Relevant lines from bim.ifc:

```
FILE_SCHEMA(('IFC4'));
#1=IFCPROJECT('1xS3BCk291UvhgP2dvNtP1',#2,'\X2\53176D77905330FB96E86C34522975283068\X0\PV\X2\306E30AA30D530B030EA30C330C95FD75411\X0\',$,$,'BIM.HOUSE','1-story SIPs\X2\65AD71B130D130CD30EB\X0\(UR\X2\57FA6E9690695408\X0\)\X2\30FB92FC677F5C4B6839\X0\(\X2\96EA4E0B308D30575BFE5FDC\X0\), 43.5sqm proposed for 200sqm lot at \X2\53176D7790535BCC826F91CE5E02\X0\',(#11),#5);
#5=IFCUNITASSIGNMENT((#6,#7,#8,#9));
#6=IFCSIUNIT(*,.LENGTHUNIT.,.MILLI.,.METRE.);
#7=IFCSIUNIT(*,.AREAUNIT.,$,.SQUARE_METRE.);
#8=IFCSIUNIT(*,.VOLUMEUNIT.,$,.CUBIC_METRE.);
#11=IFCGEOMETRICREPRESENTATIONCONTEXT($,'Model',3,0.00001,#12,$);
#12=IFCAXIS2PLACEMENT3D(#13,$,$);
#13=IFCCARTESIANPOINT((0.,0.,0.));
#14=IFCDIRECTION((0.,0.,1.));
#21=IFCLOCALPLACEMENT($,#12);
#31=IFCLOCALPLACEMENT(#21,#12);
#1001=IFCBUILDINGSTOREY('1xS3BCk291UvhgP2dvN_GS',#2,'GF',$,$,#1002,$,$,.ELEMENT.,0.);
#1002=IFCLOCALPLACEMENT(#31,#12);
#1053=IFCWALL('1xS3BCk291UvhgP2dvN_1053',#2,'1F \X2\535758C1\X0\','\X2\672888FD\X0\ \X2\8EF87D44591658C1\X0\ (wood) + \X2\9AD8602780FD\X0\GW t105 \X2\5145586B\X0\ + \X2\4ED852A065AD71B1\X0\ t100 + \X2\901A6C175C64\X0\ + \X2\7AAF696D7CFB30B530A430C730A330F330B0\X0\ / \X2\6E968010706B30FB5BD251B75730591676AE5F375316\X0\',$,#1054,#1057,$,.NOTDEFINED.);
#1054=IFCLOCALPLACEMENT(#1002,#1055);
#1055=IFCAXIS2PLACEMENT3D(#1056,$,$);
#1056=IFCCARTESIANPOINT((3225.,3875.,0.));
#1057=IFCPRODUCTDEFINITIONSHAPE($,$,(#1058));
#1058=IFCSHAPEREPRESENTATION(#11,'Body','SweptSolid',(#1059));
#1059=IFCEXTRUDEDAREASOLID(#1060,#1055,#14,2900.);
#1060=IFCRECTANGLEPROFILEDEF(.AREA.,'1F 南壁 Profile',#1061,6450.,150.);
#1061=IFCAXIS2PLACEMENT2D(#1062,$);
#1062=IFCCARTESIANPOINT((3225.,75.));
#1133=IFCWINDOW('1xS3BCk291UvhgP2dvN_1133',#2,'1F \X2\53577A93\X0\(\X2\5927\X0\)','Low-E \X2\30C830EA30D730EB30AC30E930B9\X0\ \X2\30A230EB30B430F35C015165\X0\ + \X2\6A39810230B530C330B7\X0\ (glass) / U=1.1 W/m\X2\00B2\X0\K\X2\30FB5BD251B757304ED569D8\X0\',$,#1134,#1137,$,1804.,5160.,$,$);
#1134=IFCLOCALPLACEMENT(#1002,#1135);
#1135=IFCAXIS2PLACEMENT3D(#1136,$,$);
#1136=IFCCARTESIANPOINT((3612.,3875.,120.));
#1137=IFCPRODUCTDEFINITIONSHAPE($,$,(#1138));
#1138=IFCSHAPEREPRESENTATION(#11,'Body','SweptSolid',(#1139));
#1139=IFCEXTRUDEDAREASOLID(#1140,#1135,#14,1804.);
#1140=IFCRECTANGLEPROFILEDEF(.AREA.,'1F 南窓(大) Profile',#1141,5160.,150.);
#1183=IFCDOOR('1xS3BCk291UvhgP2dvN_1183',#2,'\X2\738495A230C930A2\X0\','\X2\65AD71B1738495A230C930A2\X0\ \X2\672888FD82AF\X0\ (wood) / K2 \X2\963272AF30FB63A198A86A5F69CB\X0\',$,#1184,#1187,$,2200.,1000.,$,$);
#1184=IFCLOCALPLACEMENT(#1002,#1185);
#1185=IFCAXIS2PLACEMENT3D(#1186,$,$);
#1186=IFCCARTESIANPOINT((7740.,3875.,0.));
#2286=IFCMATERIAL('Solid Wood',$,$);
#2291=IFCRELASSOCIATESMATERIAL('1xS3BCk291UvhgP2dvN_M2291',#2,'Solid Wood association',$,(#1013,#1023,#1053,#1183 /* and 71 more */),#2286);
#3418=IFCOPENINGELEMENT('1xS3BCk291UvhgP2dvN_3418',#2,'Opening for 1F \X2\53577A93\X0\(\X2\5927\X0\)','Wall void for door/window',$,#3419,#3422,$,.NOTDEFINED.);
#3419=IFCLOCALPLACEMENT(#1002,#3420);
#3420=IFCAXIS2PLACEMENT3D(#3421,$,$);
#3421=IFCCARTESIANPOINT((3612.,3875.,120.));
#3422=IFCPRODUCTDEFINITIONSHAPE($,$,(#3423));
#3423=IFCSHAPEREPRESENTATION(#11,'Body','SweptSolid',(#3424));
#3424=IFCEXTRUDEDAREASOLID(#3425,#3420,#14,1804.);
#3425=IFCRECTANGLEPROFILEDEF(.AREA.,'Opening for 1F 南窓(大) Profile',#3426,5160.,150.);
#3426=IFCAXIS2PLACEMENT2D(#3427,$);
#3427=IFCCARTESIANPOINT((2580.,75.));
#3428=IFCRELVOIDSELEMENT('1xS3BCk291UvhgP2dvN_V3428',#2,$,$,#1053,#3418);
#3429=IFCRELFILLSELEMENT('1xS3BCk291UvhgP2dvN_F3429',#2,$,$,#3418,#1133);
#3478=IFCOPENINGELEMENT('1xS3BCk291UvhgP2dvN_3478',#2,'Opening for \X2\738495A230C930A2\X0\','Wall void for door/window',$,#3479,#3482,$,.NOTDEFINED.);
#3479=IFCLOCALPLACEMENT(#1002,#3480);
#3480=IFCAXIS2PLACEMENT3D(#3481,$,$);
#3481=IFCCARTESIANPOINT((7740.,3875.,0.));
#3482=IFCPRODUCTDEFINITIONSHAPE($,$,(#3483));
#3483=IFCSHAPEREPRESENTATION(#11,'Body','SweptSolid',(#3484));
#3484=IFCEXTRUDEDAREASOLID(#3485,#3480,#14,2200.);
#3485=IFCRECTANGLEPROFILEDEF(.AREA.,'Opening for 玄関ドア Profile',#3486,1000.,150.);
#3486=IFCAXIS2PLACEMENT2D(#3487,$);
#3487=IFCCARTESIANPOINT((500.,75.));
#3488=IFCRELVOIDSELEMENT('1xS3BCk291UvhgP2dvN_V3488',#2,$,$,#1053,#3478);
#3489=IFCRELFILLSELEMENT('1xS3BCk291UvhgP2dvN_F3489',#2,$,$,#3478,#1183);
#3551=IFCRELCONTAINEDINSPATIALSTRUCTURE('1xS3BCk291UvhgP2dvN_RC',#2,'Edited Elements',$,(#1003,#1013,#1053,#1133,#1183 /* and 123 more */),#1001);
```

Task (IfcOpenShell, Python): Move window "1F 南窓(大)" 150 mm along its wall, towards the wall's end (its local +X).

```python
import ifcopenshell
import ifcopenshell.api.geometry
import ifcopenshell.util.placement
import ifcopenshell.util.unit

model = ifcopenshell.open("bim.ifc")
unit_scale = ifcopenshell.util.unit.calculate_unit_scale(model)

window = model.by_id(1133)
opening = window.FillsVoids[0].RelatingOpeningElement
wall = opening.VoidsElements[0].RelatingBuildingElement

wall_matrix = ifcopenshell.util.placement.get_local_placement(wall.ObjectPlacement)
shift = wall_matrix[:3, 0] * 0.15 / unit_scale
before = ifcopenshell.util.placement.get_local_placement(window.ObjectPlacement)[:3, 3].copy()

# The window is not placed relative to its opening, so move both.
for product in (opening, window):
    matrix = ifcopenshell.util.placement.get_local_placement(product.ObjectPlacement)
    matrix[:3, 3] += shift
    ifcopenshell.api.geometry.edit_object_placement(model, product=product, matrix=matrix, is_si=False)

after = ifcopenshell.util.placement.get_local_placement(window.ObjectPlacement)[:3, 3]
print("window moved by", (after - before).round(3) + 0.0)

model.write("bim_edited.ifc")
```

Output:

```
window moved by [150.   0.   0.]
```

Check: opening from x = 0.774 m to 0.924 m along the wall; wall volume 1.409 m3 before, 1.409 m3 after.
